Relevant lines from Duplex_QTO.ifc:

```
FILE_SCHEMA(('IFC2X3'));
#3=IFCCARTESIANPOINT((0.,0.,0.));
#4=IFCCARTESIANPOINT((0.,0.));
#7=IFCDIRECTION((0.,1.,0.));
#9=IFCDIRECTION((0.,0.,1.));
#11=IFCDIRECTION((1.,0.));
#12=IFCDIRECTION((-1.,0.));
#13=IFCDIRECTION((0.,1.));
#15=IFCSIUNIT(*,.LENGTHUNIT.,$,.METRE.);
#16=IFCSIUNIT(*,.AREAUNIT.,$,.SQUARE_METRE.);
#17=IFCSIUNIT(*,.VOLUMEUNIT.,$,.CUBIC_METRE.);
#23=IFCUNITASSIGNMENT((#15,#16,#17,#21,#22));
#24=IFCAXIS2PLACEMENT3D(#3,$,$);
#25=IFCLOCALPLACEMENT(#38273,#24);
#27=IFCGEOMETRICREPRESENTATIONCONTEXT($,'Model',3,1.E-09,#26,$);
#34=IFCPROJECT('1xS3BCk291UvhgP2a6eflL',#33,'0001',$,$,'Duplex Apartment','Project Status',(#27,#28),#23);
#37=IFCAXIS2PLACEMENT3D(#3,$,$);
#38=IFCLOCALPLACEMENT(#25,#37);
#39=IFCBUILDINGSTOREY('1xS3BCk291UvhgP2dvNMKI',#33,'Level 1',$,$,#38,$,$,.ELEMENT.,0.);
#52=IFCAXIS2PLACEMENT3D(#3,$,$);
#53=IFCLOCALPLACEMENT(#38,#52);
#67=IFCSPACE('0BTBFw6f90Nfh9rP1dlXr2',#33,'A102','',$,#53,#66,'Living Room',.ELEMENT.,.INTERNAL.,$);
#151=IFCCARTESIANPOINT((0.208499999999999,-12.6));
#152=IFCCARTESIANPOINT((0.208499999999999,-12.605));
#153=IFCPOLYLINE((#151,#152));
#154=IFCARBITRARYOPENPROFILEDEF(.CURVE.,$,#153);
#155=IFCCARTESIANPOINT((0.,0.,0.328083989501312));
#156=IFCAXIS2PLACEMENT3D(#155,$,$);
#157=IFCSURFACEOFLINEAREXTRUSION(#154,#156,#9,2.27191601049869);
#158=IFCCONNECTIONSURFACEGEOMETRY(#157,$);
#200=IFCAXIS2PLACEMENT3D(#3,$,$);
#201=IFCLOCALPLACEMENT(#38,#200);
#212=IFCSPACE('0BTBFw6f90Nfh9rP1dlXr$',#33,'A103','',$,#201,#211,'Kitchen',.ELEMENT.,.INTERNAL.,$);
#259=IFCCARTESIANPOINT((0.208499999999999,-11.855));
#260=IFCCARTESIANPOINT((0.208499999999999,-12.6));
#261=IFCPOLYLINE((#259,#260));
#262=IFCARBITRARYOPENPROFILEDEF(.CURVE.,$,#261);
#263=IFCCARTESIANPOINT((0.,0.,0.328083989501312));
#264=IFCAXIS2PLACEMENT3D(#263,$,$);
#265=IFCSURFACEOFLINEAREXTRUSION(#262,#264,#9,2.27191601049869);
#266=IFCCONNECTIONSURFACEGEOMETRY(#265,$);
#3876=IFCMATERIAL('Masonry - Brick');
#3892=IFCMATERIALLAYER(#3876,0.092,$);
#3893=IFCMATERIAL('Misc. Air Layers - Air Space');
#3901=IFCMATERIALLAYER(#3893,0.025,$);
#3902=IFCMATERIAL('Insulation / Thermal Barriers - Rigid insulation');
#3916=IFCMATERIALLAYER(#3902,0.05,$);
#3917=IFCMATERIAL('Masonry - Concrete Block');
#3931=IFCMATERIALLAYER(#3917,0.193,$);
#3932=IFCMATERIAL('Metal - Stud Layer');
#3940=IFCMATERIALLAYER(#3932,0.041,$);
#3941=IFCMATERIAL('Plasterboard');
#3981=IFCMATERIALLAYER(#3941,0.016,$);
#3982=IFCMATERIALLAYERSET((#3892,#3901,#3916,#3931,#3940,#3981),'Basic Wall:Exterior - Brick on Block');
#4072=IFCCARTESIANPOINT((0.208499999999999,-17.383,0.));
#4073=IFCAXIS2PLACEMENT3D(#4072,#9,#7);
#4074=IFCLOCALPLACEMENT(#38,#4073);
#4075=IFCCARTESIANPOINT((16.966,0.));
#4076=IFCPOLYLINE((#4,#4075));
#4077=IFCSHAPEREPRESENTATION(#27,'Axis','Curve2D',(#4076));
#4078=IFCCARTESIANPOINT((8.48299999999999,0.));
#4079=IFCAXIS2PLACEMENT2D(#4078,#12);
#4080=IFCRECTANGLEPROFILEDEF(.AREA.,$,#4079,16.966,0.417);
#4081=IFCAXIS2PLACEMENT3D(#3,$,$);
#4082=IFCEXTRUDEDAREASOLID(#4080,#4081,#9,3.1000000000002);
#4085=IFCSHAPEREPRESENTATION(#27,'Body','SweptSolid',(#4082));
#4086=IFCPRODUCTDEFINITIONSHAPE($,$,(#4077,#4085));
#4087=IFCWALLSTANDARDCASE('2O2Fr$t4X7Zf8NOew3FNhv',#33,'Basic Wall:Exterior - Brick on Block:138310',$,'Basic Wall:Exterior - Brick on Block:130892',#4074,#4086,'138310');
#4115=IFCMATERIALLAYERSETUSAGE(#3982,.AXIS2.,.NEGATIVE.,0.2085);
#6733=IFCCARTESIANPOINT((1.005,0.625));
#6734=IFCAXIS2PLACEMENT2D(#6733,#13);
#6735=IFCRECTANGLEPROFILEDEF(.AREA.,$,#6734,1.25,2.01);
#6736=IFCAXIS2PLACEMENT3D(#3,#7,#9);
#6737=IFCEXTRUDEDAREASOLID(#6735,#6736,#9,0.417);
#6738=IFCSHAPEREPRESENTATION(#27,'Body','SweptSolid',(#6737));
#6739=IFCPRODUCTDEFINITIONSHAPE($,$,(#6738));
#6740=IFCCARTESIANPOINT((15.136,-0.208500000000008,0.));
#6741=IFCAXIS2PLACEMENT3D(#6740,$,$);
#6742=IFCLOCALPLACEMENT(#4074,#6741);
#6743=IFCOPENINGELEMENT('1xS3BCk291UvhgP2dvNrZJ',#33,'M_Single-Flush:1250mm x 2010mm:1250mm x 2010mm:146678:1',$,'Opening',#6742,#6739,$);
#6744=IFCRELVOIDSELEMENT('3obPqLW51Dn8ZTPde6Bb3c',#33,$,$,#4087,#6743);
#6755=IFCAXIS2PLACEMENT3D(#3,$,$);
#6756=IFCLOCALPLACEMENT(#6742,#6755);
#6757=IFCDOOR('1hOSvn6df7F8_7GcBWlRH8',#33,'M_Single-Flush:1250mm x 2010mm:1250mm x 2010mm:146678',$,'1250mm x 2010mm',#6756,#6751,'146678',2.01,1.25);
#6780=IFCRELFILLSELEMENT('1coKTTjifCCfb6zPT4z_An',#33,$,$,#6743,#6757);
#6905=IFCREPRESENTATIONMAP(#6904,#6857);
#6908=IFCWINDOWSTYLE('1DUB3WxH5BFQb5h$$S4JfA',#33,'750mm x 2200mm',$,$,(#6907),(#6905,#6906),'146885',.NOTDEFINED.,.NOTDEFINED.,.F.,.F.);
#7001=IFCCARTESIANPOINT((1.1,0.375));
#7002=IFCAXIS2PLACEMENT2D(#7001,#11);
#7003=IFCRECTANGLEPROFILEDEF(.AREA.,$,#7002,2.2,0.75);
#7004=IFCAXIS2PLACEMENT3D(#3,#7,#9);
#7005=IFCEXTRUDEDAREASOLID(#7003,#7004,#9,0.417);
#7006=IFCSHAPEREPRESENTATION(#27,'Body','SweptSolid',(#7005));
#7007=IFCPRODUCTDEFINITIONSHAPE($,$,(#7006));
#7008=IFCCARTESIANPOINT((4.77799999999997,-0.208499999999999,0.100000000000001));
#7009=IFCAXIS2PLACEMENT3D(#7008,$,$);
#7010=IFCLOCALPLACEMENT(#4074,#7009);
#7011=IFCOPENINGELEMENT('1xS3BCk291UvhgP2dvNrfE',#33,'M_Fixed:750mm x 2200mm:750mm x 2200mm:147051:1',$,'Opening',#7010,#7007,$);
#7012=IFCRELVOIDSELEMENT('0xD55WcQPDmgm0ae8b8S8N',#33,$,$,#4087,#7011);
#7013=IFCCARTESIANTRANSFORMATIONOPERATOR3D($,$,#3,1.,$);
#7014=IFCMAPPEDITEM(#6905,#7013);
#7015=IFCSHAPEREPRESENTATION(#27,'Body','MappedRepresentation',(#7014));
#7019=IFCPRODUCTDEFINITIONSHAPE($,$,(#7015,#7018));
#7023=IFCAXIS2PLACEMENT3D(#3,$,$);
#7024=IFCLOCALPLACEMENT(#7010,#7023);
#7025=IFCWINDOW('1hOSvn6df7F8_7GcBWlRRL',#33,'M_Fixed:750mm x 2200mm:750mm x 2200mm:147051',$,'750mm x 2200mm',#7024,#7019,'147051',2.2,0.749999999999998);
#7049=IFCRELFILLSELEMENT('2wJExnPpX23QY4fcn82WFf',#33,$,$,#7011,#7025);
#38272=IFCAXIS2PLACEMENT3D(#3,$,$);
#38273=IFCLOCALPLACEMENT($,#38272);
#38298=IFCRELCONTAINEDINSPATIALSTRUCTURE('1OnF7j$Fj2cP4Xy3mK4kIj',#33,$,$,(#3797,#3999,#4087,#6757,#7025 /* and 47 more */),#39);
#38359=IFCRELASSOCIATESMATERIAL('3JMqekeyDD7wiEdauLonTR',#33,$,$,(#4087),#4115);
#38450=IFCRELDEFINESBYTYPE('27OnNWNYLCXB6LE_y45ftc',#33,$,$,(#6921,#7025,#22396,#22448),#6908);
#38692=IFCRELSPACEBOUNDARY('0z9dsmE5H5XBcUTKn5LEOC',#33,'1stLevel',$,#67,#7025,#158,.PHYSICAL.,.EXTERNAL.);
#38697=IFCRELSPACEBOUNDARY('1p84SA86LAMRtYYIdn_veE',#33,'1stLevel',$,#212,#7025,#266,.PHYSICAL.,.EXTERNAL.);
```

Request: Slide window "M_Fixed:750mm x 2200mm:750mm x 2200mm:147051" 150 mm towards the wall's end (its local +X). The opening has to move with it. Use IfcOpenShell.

```python
import numpy as np
import ifcopenshell
import ifcopenshell.api.geometry
import ifcopenshell.util.placement
import ifcopenshell.util.unit

model = ifcopenshell.open("Duplex_QTO.ifc")
unit_scale = ifcopenshell.util.unit.calculate_unit_scale(model)

window = model.by_guid("1hOSvn6df7F8_7GcBWlRRL")
opening = window.FillsVoids[0].RelatingOpeningElement
wall = opening.VoidsElements[0].RelatingBuildingElement

wall_matrix = ifcopenshell.util.placement.get_local_placement(wall.ObjectPlacement)
shift = wall_matrix[:3, 0] * 0.15 / unit_scale
before = ifcopenshell.util.placement.get_local_placement(window.ObjectPlacement)[:3, 3].copy()

# The window is placed relative to its opening, so it follows when the opening moves.
matrix = ifcopenshell.util.placement.get_local_placement(opening.ObjectPlacement)
matrix[:3, 3] += shift
ifcopenshell.api.geometry.edit_object_placement(
    model, product=opening, matrix=matrix, is_si=False, should_transform_children=True
)

# Space boundary surfaces are stored in each space's coordinates; move them too.
for rel in window.ProvidesBoundaries:
    if not rel.ConnectionGeometry:
        continue
    surface = rel.ConnectionGeometry.SurfaceOnRelatingElement
    space_matrix = ifcopenshell.util.placement.get_local_placement(rel.RelatingSpace.ObjectPlacement)
    point = np.array(surface.Position.Location.Coordinates) + space_matrix[:3, :3].T @ shift
    surface.Position = model.createIfcAxis2Placement3D(
        model.createIfcCartesianPoint(point.tolist()), surface.Position.Axis, surface.Position.RefDirection
    )

after = ifcopenshell.util.placement.get_local_placement(window.ObjectPlacement)[:3, 3]
print("window moved by", (after - before).round(3) + 0.0)

model.write("Duplex_QTO_rev.ifc")
```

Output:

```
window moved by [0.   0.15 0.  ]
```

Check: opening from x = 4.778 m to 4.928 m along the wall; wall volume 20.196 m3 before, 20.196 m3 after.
